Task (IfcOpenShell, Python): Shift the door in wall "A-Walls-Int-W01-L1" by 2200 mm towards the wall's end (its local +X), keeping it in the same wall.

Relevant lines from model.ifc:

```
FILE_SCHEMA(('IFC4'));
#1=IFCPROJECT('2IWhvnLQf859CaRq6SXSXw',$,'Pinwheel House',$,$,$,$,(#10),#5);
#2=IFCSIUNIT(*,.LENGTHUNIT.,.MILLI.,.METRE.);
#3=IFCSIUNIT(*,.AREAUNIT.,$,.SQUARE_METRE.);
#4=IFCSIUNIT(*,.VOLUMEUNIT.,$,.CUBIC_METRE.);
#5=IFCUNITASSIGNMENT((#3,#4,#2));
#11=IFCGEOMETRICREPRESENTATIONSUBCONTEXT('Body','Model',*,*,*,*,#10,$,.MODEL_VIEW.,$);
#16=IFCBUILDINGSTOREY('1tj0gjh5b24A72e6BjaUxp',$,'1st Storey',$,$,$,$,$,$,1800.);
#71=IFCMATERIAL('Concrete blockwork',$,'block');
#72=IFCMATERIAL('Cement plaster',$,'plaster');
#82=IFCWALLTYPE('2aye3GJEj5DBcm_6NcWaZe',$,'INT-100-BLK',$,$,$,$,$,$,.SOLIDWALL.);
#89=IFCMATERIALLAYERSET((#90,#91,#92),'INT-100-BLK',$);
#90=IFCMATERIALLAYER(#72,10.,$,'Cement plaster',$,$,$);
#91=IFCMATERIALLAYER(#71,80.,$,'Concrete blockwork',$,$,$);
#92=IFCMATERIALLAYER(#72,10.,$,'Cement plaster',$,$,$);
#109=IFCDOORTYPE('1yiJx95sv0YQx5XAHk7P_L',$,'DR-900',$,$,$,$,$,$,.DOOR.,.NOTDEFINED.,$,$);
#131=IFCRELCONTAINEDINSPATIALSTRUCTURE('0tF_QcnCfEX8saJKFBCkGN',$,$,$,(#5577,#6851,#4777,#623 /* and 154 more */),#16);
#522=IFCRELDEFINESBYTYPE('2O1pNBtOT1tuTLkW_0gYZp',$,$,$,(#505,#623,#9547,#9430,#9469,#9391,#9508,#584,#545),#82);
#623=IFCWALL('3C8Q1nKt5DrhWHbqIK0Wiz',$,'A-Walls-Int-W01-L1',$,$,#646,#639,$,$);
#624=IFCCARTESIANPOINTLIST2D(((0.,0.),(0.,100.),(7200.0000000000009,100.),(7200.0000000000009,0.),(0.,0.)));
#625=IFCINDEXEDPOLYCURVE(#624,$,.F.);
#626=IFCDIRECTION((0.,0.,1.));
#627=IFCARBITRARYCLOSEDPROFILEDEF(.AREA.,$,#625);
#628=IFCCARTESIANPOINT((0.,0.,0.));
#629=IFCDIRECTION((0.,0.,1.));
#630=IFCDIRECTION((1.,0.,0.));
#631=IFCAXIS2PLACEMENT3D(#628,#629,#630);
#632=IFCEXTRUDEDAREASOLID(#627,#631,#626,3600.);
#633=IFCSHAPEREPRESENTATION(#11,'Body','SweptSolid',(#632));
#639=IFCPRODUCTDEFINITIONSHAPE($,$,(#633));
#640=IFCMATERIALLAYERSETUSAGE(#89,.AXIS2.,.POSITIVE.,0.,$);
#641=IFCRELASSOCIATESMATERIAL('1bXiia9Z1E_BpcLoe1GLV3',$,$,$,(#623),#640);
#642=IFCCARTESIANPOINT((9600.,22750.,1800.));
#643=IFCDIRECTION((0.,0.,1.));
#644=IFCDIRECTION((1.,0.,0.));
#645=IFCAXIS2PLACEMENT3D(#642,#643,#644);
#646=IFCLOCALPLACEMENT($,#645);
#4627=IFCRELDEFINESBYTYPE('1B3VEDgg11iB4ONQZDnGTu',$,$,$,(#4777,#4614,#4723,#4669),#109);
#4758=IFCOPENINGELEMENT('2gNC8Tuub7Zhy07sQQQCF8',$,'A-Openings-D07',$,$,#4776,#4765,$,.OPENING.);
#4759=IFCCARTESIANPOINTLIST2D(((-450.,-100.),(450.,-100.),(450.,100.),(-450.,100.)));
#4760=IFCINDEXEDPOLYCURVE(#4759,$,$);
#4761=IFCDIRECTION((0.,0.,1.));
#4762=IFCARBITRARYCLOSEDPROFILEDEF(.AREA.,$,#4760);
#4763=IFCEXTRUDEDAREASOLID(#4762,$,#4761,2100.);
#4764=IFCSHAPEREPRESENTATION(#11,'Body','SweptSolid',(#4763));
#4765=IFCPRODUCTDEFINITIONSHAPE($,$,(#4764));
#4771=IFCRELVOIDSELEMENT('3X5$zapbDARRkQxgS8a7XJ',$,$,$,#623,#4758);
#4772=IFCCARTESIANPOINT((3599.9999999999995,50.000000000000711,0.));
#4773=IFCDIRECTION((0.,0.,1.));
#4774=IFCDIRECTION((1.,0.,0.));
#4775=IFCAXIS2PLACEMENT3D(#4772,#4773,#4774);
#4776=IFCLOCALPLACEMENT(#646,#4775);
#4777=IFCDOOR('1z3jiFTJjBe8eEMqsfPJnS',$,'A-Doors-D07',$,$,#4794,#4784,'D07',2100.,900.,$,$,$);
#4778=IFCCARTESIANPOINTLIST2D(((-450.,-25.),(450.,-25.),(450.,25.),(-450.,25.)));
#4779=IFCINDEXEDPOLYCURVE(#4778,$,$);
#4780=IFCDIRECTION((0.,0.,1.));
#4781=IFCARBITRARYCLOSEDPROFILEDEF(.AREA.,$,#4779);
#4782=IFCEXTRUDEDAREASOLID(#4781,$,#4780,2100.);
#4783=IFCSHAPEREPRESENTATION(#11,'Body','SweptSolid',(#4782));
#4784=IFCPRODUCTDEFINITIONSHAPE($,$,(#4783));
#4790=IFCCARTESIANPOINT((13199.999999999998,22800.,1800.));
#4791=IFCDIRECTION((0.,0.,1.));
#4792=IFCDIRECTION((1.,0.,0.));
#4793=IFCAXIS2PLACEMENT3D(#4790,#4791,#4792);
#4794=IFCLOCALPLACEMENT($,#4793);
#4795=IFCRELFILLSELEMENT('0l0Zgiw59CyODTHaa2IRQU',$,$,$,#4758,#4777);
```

```python
import ifcopenshell
import ifcopenshell.api.geometry
import ifcopenshell.util.placement
import ifcopenshell.util.unit

model = ifcopenshell.open("model.ifc")
unit_scale = ifcopenshell.util.unit.calculate_unit_scale(model)

door = model.by_guid("1z3jiFTJjBe8eEMqsfPJnS")
opening = door.FillsVoids[0].RelatingOpeningElement
wall = opening.VoidsElements[0].RelatingBuildingElement

wall_matrix = ifcopenshell.util.placement.get_local_placement(wall.ObjectPlacement)
shift = wall_matrix[:3, 0] * 2.2 / unit_scale
before = ifcopenshell.util.placement.get_local_placement(door.ObjectPlacement)[:3, 3].copy()

# The door is not placed relative to its opening, so move both.
for product in (opening, door):
    matrix = ifcopenshell.util.placement.get_local_placement(product.ObjectPlacement)
    matrix[:3, 3] += shift
    ifcopenshell.api.geometry.edit_object_placement(model, product=product, matrix=matrix, is_si=False)

after = ifcopenshell.util.placement.get_local_placement(door.ObjectPlacement)[:3, 3]
print("door moved by", (after - before).round(3) + 0.0)

model.write("model_edited.ifc")
```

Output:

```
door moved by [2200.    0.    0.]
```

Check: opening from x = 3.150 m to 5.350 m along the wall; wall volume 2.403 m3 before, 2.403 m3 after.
